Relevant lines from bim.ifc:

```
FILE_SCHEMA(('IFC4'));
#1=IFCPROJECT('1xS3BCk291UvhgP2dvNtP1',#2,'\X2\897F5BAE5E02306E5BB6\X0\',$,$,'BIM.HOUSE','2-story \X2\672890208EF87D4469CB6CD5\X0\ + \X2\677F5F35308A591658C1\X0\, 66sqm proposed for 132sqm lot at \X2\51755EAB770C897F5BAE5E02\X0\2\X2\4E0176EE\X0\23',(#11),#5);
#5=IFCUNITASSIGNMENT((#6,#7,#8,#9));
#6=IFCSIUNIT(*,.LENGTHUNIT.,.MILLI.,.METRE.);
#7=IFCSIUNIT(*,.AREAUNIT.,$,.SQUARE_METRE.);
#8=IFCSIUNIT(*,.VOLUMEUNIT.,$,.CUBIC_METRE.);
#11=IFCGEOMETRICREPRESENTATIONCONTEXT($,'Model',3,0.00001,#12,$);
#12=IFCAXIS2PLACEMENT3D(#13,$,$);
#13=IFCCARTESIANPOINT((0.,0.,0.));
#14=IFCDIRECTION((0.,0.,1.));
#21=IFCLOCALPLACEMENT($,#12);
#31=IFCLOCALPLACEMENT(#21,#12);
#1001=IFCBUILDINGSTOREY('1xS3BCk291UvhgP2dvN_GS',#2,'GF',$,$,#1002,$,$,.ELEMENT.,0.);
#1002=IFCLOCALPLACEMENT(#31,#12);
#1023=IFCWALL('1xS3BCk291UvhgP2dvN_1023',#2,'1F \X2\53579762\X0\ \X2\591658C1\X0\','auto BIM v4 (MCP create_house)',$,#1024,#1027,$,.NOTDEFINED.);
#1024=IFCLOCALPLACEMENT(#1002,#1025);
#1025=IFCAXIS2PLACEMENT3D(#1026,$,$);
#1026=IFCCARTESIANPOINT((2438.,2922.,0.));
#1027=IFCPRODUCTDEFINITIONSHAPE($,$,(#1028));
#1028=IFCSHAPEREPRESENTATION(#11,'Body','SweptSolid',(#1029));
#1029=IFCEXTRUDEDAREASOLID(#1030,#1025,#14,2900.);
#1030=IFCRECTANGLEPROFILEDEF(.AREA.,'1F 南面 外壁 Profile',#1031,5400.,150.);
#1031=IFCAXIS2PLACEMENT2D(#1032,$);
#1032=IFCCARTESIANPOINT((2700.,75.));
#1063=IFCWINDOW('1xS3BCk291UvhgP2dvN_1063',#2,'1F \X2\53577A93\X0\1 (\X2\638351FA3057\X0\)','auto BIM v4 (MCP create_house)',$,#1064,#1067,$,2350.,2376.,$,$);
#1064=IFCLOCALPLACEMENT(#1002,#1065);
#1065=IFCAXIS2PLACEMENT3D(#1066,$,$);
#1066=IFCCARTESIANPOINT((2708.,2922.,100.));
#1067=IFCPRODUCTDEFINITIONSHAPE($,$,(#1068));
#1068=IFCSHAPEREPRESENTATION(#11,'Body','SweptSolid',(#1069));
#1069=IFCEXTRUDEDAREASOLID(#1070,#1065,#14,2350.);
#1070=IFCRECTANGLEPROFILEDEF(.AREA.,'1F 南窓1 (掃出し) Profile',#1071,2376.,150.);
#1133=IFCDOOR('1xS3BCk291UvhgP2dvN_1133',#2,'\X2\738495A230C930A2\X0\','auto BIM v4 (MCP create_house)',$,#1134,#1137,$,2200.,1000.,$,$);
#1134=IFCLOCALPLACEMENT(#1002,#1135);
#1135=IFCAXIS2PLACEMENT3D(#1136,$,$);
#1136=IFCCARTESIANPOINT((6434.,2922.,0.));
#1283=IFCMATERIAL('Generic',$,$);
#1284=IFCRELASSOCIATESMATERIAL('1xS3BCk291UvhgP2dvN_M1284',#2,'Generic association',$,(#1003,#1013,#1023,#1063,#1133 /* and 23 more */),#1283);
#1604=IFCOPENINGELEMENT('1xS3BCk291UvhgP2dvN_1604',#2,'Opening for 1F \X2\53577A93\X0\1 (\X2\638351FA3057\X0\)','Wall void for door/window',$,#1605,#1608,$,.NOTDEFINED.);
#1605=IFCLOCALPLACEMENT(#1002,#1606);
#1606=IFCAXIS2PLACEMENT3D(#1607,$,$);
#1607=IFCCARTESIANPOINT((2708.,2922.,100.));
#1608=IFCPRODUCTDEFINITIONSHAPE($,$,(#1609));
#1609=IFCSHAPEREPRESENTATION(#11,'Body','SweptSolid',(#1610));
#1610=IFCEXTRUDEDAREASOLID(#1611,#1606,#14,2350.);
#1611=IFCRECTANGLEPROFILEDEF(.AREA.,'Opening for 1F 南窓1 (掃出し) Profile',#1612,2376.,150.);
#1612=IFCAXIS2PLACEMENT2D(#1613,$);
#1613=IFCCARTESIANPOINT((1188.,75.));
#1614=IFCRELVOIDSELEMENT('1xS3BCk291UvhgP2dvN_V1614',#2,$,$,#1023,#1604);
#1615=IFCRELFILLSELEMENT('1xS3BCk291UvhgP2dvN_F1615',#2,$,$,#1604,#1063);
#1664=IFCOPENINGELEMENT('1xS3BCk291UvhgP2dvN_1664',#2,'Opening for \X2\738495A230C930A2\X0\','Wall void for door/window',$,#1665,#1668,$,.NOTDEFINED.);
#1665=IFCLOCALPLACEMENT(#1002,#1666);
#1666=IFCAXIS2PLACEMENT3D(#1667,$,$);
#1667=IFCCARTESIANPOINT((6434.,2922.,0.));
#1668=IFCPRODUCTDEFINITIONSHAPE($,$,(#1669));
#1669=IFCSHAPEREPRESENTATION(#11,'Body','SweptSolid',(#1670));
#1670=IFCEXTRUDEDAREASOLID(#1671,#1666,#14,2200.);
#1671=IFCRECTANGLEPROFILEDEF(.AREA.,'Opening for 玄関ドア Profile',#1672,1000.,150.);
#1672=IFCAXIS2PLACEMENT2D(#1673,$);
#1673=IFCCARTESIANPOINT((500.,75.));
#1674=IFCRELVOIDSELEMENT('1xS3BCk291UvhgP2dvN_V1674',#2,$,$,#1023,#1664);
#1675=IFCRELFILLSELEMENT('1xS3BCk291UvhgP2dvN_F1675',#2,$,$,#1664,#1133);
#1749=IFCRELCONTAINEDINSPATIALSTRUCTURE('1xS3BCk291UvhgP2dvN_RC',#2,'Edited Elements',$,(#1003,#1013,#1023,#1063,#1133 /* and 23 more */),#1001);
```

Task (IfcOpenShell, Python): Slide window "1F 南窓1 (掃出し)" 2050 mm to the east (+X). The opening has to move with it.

```python
import ifcopenshell
import ifcopenshell.api.geometry
import ifcopenshell.util.placement

model = ifcopenshell.open("bim.ifc")

window = model.by_id(1063)
opening = window.FillsVoids[0].RelatingOpeningElement
wall = opening.VoidsElements[0].RelatingBuildingElement

wall_matrix = ifcopenshell.util.placement.get_local_placement(wall.ObjectPlacement)
shift = wall_matrix[:3, 0] * 2050.0
before = ifcopenshell.util.placement.get_local_placement(window.ObjectPlacement)[:3, 3].copy()

# The window is not placed relative to its opening, so move both.
for product in (opening, window):
    matrix = ifcopenshell.util.placement.get_local_placement(product.ObjectPlacement)
    matrix[:3, 3] += shift
    ifcopenshell.api.geometry.edit_object_placement(model, product=product, matrix=matrix, is_si=False)

after = ifcopenshell.util.placement.get_local_placement(window.ObjectPlacement)[:3, 3]
print("window moved by", (after - before).round(3) + 0.0)

model.write("bim-out.ifc")
```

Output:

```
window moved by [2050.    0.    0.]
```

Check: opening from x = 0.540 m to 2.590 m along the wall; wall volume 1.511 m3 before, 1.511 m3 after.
